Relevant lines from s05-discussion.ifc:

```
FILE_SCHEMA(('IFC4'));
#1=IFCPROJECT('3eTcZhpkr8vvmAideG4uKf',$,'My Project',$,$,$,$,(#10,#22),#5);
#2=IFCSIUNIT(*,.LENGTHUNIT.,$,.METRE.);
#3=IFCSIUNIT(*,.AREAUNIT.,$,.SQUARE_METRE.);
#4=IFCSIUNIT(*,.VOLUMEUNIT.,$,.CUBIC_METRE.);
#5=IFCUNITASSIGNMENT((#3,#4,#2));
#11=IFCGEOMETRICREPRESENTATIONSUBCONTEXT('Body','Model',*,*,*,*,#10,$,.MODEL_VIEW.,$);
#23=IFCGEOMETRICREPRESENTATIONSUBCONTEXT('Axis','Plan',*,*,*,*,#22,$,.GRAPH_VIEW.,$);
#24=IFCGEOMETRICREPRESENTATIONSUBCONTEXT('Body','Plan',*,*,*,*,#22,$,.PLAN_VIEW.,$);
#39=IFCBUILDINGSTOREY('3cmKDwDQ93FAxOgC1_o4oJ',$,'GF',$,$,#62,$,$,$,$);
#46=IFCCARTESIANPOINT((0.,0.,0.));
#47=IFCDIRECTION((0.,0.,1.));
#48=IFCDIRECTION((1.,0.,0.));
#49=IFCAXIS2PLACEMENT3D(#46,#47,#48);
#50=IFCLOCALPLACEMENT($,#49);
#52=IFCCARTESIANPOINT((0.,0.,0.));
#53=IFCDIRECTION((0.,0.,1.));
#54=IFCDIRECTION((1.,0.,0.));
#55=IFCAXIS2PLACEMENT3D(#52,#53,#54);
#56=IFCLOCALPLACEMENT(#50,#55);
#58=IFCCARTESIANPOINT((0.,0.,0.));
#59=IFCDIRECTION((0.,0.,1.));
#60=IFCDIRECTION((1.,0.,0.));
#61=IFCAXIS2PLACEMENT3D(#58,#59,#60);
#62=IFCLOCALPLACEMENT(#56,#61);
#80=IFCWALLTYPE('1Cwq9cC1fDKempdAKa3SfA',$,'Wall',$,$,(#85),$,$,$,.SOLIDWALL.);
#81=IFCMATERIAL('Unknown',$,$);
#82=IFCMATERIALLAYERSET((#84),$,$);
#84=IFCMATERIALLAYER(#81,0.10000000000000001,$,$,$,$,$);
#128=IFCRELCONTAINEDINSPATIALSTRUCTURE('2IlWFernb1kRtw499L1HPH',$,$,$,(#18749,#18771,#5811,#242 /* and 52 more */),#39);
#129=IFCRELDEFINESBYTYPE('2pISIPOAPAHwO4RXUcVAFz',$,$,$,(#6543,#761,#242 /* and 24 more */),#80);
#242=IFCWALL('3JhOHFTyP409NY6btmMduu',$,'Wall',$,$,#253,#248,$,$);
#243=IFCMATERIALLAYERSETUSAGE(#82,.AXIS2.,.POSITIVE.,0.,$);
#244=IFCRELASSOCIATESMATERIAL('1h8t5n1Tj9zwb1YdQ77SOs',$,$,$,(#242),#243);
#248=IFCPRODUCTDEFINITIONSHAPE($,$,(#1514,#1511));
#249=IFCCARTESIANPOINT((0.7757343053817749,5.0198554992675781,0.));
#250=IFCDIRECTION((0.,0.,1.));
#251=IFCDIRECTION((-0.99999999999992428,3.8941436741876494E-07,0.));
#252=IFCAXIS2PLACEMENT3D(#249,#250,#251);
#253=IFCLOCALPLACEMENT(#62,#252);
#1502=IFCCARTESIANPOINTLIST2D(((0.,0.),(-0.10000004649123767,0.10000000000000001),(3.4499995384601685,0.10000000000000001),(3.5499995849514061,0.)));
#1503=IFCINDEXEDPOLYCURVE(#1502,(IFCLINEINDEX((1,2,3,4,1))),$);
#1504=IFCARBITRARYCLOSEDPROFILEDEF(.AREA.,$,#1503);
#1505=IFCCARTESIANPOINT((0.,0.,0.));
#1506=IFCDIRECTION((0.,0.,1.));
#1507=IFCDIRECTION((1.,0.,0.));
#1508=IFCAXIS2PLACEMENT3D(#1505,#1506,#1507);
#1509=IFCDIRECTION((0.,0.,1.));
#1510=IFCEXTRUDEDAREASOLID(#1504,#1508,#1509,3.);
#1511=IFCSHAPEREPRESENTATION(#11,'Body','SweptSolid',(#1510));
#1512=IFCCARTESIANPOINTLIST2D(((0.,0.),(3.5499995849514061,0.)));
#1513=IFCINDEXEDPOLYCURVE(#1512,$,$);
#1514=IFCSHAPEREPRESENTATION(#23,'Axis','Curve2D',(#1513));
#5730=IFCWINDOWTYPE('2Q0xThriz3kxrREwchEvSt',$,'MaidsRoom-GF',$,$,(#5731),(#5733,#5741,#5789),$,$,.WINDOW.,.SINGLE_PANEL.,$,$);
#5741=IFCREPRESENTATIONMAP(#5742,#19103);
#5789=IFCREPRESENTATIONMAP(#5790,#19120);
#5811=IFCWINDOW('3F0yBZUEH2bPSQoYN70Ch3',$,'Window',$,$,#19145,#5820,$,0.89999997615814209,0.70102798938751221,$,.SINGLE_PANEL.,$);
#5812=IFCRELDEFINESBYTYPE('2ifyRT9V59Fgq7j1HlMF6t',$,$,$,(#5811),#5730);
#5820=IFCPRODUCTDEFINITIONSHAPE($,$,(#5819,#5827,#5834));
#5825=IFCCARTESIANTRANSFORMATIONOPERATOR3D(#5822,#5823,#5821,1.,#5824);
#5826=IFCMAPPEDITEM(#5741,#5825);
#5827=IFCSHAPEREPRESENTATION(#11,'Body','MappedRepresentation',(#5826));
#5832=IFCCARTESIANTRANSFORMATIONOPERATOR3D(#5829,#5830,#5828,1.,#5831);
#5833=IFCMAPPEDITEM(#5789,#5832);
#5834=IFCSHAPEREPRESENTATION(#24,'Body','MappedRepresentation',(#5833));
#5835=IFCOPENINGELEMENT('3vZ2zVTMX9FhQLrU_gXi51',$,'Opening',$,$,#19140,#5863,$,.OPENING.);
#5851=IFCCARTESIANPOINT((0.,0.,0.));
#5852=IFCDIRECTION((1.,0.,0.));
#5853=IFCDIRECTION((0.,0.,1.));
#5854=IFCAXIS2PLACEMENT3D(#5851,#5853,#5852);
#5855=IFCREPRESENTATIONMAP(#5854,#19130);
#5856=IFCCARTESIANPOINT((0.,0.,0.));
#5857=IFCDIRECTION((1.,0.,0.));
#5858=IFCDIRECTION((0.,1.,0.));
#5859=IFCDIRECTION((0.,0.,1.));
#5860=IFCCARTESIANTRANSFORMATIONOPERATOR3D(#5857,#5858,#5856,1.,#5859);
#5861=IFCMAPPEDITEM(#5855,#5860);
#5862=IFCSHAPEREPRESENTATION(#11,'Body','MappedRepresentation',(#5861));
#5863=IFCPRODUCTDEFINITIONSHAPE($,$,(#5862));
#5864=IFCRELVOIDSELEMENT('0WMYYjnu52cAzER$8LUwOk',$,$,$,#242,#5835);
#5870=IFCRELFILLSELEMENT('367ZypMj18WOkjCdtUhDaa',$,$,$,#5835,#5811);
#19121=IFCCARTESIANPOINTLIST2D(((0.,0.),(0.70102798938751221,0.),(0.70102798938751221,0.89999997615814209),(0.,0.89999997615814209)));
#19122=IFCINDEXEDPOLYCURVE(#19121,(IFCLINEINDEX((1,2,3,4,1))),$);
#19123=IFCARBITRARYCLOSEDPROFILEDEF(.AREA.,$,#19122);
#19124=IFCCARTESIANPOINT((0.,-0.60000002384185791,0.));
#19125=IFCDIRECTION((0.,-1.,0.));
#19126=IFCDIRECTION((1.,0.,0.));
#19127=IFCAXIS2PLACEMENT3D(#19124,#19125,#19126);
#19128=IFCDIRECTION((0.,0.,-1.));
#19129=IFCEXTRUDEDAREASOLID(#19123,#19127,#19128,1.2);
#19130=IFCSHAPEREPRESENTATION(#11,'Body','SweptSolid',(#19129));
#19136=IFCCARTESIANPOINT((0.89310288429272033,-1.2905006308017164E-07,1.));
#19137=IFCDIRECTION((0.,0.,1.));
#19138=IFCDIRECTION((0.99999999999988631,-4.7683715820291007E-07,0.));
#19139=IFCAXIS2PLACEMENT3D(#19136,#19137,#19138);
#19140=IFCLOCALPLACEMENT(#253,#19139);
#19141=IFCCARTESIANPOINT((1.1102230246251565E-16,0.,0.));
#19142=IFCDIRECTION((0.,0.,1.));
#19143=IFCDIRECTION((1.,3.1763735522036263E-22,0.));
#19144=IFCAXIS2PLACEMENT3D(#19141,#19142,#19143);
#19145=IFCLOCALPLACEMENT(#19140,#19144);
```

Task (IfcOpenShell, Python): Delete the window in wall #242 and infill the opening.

```python
import ifcopenshell
import ifcopenshell.api.feature
import ifcopenshell.api.root
import ifcopenshell.geom
import ifcopenshell.util.shape

model = ifcopenshell.open("s05-discussion.ifc")
settings = ifcopenshell.geom.settings()


def volume(element):
    """Net volume in cubic metres, openings subtracted."""
    shape = ifcopenshell.geom.create_shape(settings, element)
    return ifcopenshell.util.shape.get_volume(shape.geometry)


window = model.by_id(5811)
opening = window.FillsVoids[0].RelatingOpeningElement
wall = opening.VoidsElements[0].RelatingBuildingElement
before = volume(wall)

ifcopenshell.api.root.remove_product(model, product=window)
ifcopenshell.api.feature.remove_feature(model, feature=opening)

after = volume(wall)

print(f"wall volume {before:.3f} -> {after:.3f} m3")

model.write("s05-discussion_edited.ifc")
```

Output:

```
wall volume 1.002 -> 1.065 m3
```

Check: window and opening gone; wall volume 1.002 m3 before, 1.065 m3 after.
